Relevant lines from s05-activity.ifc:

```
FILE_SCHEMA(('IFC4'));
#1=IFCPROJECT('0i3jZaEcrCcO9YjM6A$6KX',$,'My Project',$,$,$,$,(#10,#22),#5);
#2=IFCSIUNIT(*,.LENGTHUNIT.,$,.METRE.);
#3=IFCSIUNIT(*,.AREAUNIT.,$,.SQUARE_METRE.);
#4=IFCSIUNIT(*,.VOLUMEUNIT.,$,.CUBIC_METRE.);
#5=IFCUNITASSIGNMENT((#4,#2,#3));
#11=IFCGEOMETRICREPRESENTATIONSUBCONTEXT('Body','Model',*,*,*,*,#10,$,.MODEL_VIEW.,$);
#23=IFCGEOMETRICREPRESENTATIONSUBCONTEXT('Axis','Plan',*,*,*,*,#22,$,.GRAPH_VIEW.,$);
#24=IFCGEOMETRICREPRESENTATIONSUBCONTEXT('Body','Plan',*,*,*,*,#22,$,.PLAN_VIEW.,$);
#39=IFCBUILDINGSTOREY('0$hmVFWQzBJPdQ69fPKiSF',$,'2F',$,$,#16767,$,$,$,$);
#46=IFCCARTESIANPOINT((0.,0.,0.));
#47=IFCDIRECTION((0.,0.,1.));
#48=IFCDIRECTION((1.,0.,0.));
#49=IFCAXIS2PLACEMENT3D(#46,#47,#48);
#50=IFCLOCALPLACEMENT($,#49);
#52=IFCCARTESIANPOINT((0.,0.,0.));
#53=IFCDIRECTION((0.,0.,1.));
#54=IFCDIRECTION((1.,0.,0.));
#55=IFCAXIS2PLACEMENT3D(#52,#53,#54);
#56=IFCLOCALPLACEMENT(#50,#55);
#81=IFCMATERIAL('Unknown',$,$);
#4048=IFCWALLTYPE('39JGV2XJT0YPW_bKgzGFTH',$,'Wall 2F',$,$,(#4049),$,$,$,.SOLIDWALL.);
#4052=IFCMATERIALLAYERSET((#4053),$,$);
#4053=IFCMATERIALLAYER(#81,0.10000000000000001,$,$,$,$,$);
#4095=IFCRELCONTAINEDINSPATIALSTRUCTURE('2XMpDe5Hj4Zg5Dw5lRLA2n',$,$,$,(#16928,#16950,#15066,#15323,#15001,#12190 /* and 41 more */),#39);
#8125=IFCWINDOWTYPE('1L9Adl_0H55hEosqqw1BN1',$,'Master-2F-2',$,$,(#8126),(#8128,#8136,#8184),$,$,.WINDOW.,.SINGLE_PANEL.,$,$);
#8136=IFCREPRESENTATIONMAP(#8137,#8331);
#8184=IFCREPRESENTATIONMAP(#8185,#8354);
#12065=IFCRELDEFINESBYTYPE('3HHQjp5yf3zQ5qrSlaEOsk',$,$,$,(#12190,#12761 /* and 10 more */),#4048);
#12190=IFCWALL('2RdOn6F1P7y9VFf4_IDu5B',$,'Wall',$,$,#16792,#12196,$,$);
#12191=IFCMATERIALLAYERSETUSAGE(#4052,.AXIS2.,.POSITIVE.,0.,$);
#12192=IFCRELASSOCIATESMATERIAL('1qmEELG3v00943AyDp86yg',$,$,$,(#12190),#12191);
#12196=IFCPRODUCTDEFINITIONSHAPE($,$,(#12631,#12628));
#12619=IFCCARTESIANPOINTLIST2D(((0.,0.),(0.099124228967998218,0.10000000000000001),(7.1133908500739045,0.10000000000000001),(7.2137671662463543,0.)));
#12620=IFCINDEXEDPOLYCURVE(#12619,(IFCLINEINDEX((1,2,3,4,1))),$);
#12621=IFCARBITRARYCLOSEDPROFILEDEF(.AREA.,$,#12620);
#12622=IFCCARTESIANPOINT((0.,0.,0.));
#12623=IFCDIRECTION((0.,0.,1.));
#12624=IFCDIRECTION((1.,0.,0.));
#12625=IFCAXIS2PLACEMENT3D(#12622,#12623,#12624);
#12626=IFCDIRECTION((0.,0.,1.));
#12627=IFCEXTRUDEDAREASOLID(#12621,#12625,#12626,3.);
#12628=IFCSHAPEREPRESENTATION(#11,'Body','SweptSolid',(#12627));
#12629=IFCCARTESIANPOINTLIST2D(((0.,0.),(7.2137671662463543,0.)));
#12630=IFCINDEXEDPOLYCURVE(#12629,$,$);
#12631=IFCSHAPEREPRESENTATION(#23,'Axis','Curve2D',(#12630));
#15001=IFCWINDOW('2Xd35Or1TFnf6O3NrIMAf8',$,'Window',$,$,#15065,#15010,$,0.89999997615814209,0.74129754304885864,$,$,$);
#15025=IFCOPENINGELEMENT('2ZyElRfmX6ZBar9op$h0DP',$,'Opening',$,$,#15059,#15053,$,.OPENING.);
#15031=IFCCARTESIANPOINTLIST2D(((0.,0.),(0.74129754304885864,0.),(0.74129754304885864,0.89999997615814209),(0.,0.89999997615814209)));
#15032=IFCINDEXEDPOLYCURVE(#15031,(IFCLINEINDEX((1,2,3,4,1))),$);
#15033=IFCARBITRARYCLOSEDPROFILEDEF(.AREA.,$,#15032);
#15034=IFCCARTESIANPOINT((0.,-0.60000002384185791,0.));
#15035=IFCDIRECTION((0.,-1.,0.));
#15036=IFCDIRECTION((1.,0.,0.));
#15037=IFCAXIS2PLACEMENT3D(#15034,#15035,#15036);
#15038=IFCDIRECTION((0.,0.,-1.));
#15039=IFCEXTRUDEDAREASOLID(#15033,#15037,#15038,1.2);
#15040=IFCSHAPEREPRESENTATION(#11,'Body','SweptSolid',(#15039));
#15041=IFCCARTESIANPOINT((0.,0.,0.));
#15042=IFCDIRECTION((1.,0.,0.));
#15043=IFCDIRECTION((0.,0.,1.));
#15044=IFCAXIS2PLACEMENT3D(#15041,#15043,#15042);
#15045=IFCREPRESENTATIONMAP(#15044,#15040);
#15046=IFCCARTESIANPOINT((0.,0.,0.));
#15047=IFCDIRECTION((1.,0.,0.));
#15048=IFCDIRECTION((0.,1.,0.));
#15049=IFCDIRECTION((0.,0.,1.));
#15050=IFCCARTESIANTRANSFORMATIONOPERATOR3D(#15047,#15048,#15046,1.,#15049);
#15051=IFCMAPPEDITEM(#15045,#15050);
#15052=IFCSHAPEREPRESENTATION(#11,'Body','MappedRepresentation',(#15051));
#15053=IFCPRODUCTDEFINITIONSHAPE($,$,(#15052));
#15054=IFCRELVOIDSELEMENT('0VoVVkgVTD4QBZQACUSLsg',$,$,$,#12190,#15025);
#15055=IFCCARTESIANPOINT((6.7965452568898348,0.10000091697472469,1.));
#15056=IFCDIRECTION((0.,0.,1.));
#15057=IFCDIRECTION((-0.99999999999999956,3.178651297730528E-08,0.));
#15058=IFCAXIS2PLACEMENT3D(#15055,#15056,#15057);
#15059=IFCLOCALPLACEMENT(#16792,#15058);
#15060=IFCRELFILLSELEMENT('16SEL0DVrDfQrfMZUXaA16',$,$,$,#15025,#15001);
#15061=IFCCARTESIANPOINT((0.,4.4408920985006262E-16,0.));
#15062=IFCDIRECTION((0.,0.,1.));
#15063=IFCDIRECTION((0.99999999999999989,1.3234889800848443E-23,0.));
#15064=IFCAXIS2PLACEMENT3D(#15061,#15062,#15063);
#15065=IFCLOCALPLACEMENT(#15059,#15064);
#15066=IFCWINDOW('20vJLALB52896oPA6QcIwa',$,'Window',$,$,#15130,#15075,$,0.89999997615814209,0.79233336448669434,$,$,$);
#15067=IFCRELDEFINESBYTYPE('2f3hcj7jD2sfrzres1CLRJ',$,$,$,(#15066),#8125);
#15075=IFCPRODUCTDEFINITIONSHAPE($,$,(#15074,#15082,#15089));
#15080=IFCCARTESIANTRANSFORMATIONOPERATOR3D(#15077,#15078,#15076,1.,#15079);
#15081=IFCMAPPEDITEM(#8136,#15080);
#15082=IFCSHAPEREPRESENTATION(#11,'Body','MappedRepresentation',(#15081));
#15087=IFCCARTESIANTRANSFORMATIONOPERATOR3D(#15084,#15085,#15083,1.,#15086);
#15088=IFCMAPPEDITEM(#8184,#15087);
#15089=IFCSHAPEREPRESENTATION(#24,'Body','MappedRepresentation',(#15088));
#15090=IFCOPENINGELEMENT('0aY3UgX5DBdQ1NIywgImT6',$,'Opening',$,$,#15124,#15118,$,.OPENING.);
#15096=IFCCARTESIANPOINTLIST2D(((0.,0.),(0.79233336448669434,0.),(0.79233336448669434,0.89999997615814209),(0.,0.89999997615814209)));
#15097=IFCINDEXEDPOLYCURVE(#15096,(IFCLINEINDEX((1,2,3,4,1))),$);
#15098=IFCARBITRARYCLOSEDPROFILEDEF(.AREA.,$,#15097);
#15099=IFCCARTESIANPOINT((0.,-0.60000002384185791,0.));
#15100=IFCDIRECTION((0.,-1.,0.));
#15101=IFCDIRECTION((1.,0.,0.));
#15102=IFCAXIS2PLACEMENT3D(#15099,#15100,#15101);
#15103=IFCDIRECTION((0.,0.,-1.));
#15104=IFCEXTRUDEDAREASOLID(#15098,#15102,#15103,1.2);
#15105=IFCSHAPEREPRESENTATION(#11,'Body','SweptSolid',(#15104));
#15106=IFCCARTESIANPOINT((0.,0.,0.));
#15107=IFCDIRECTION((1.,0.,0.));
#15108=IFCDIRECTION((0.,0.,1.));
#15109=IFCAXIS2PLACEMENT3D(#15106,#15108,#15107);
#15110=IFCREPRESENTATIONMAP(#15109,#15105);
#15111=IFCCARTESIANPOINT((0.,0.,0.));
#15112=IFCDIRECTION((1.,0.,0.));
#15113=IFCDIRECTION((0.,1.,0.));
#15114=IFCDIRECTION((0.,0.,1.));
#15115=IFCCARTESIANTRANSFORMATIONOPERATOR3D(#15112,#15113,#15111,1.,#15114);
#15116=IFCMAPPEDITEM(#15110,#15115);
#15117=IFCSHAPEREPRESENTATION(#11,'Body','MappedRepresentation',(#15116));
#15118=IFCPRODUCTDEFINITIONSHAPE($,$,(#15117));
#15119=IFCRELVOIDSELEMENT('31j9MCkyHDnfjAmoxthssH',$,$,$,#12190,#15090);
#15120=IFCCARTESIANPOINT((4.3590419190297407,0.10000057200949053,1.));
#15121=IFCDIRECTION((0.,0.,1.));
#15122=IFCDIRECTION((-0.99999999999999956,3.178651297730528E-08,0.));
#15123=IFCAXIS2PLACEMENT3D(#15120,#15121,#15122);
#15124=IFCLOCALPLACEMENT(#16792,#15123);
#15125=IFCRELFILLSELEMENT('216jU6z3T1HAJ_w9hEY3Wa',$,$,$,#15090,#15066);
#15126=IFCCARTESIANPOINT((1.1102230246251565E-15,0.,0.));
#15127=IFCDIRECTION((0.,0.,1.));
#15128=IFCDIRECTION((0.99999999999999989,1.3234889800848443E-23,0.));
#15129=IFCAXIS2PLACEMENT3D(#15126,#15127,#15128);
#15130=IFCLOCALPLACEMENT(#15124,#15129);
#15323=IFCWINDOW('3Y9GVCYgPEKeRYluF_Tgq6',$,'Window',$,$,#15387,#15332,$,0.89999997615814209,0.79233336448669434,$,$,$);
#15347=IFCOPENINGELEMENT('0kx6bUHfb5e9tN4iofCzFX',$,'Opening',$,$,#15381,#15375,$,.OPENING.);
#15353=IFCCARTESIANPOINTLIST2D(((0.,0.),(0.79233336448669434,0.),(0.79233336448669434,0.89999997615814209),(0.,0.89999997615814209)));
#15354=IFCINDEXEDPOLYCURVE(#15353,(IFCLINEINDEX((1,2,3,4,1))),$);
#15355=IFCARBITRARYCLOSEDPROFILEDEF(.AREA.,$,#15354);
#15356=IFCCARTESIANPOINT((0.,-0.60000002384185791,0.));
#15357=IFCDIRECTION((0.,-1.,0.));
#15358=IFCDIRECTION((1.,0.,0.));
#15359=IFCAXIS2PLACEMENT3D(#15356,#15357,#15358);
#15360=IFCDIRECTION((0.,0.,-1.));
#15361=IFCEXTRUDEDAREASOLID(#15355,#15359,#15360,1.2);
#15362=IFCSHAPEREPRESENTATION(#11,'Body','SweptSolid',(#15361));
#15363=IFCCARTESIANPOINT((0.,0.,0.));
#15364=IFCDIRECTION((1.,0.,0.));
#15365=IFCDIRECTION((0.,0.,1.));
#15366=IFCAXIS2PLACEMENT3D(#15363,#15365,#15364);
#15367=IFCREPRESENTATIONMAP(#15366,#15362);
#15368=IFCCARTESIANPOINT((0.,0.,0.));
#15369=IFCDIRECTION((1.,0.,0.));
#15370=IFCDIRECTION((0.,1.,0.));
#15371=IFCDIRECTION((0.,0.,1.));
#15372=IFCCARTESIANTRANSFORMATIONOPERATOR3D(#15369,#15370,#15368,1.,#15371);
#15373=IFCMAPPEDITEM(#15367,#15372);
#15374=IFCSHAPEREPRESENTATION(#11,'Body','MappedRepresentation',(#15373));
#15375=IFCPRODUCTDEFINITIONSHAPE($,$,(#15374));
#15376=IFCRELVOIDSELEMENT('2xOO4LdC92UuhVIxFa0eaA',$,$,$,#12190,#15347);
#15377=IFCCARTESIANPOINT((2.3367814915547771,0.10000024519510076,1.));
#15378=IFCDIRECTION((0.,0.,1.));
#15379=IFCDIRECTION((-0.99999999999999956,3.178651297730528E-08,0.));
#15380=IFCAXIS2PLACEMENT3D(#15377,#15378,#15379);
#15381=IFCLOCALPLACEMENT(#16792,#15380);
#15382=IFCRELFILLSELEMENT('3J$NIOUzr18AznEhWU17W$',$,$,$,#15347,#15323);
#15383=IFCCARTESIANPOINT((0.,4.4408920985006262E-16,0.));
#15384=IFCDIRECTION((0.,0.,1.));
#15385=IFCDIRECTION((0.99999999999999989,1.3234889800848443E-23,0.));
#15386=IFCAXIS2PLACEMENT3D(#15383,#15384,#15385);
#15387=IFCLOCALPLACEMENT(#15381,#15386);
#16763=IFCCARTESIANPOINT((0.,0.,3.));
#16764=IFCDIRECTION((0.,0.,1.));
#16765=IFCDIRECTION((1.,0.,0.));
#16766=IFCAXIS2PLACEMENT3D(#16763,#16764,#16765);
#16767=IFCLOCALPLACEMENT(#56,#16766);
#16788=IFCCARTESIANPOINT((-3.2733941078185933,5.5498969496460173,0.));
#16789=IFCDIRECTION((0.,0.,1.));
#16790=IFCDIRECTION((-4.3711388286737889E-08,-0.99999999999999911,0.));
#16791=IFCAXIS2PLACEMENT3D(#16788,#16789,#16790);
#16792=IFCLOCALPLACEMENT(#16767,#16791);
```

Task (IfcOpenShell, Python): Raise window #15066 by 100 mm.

```python
import numpy as np
import ifcopenshell
import ifcopenshell.api.geometry
import ifcopenshell.util.placement
import ifcopenshell.util.unit

model = ifcopenshell.open("s05-activity.ifc")
unit_scale = ifcopenshell.util.unit.calculate_unit_scale(model)

window = model.by_guid("20vJLALB52896oPA6QcIwa")
opening = window.FillsVoids[0].RelatingOpeningElement
dz = 0.1 / unit_scale

shift = np.array([0.0, 0.0, dz])
# The window is placed relative to its opening, so it follows when the opening moves.
matrix = ifcopenshell.util.placement.get_local_placement(opening.ObjectPlacement)
matrix[:3, 3] += shift
ifcopenshell.api.geometry.edit_object_placement(
    model, product=opening, matrix=matrix, is_si=False, should_transform_children=True
)

print(f"moved by {dz * unit_scale:+.3f} m")

model.write("s05-activity_rev.ifc")
```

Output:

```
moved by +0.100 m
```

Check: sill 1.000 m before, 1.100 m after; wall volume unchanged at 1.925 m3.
